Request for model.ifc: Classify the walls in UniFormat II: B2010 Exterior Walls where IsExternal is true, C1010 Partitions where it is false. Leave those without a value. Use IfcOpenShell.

First a look at what the model holds.

```python
import ifcopenshell
import ifcopenshell.util.element

model = ifcopenshell.open("model.ifc")
print(model.schema)
print("classifications:", [c.Name for c in model.by_type("IfcClassification")])
values = [ifcopenshell.util.element.get_pset(e, "Pset_WallCommon", "IsExternal") for e in model.by_type("IfcWall")]
for value in (True, False, None):
    print("IsExternal", value, values.count(value))
```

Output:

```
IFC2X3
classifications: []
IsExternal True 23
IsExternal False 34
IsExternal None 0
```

```python
import ifcopenshell
import ifcopenshell.api.classification
import ifcopenshell.util.element

model = ifcopenshell.open("model.ifc")

# IFC2X3 requires Source and Edition and has no link from the project to the system.
system = model.create_entity("IfcClassification", Source="ASTM", Edition="E1557", Name="UniFormat II")

walls = model.by_type("IfcWall")
external = {e: ifcopenshell.util.element.get_pset(e, "Pset_WallCommon", "IsExternal") for e in walls}
for flag, code, name in ((True, "B2010", "Exterior Walls"), (False, "C1010", "Partitions")):
    products = [e for e in walls if external[e] is flag]
    ifcopenshell.api.classification.add_reference(
        model, products=products, classification=system, identification=code, name=name
    )
    print(code, len(products))

model.write("model_rev.ifc")
```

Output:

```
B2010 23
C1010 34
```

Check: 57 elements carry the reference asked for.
